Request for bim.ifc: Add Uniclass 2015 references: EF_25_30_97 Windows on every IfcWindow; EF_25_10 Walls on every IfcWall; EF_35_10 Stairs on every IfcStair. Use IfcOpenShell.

First a look at what the model holds.

```python
import ifcopenshell

model = ifcopenshell.open("bim.ifc")
print(model.schema)
print("classifications:", [c.Name for c in model.by_type("IfcClassification")])
for ifc_class in ("IfcDoor", "IfcRoof", "IfcStair", "IfcWall", "IfcWindow"):
    print(ifc_class, len(model.by_type(ifc_class)))
```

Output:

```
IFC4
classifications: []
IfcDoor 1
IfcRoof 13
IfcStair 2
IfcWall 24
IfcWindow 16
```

```python
import ifcopenshell
import ifcopenshell.api.classification

model = ifcopenshell.open("bim.ifc")

system = ifcopenshell.api.classification.add_classification(model, classification="Uniclass 2015")

codes = {
    "IfcWindow": ("EF_25_30_97", "Windows"),
    "IfcWall": ("EF_25_10", "Walls"),
    "IfcStair": ("EF_35_10", "Stairs"),
}
for ifc_class, (code, name) in codes.items():
    products = model.by_type(ifc_class)
    ifcopenshell.api.classification.add_reference(
        model, products=products, classification=system, identification=code, name=name
    )
    print(code, len(products))

model.write("bim_v2.ifc")
```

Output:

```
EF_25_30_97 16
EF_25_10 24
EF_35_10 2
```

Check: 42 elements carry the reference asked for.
